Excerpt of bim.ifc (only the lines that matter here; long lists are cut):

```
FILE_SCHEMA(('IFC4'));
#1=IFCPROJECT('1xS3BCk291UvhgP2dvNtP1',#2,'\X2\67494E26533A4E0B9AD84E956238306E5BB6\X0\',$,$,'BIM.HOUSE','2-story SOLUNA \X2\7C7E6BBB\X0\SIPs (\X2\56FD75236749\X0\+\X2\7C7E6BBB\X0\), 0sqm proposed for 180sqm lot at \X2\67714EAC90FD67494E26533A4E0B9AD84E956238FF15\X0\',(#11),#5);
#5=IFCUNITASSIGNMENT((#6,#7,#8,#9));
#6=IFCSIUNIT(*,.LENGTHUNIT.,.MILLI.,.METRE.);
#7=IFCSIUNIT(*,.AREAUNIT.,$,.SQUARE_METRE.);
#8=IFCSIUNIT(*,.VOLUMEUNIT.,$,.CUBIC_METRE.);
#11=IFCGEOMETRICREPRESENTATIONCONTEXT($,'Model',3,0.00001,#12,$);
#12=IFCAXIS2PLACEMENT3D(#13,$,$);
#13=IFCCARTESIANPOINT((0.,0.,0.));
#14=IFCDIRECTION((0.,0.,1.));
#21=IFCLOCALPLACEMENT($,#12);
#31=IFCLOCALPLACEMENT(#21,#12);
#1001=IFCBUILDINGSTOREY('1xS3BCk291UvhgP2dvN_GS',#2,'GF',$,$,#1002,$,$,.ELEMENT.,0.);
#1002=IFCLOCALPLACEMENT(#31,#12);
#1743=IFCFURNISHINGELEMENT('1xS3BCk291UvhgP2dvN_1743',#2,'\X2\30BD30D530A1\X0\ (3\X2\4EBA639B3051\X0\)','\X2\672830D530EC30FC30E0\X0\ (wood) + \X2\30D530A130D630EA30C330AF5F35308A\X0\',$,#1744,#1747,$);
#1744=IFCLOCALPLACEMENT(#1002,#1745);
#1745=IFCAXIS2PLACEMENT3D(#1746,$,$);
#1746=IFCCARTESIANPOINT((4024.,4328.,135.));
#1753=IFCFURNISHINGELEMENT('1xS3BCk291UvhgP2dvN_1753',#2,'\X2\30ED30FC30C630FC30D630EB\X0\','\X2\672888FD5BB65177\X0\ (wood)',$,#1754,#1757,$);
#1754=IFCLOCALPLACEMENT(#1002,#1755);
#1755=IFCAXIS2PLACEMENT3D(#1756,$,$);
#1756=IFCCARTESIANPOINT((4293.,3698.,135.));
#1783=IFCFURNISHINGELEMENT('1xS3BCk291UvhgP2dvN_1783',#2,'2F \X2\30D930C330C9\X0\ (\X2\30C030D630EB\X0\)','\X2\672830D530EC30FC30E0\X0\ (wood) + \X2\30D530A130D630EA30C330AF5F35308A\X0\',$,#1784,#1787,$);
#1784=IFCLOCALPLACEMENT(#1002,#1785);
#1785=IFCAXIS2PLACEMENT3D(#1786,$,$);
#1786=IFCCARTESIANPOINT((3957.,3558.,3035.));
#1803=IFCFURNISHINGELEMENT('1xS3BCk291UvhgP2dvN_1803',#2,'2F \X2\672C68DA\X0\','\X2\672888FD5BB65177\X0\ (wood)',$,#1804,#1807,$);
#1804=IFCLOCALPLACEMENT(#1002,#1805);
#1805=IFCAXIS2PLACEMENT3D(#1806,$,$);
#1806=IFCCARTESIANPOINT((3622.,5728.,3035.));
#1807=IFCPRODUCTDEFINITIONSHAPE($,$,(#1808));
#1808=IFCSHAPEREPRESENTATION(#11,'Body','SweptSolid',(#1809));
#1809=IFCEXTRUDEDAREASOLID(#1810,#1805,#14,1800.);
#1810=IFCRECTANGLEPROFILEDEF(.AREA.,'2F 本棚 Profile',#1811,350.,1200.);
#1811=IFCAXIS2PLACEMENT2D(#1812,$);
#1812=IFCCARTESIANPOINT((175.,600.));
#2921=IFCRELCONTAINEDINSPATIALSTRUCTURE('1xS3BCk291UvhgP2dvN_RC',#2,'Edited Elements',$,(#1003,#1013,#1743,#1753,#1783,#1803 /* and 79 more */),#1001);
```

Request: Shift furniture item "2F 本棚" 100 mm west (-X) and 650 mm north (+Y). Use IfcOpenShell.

```python
import ifcopenshell
import ifcopenshell.api.geometry
import ifcopenshell.util.placement

model = ifcopenshell.open("bim.ifc")

item = model.by_guid("1xS3BCk291UvhgP2dvN_1803")
matrix = ifcopenshell.util.placement.get_local_placement(item.ObjectPlacement)
matrix[0, 3] -= 100.0
matrix[1, 3] += 650.0
ifcopenshell.api.geometry.edit_object_placement(model, product=item, matrix=matrix, is_si=False)

print(ifcopenshell.util.placement.get_local_placement(item.ObjectPlacement).round(3) + 0.0)

model.write("bim_updated.ifc")
```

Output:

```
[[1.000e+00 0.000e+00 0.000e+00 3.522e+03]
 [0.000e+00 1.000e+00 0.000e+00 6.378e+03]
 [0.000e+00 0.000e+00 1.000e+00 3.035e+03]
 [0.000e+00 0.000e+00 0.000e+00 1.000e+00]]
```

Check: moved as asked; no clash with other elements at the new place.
